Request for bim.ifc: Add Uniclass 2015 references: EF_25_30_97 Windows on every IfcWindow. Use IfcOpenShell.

First a look at what the model holds.

```python
import ifcopenshell

model = ifcopenshell.open("bim.ifc")
print(model.schema)
print("classifications:", [c.Name for c in model.by_type("IfcClassification")])
for ifc_class in ("IfcDoor", "IfcRoof", "IfcStair", "IfcWall", "IfcWindow"):
    print(ifc_class, len(model.by_type(ifc_class)))
```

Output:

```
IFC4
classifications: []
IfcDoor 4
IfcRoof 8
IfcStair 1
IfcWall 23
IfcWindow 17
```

```python
import ifcopenshell
import ifcopenshell.api.classification

model = ifcopenshell.open("bim.ifc")

system = ifcopenshell.api.classification.add_classification(model, classification="Uniclass 2015")

codes = {
    "IfcWindow": ("EF_25_30_97", "Windows"),
}
for ifc_class, (code, name) in codes.items():
    products = model.by_type(ifc_class)
    ifcopenshell.api.classification.add_reference(
        model, products=products, classification=system, identification=code, name=name
    )
    print(code, len(products))

model.write("bim_edited.ifc")
```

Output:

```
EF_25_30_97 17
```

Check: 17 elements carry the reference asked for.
